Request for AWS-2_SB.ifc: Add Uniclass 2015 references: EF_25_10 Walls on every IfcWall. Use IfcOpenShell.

First a look at what the model holds.

```python
import ifcopenshell

model = ifcopenshell.open("AWS-2_SB.ifc")
print(model.schema)
print("classifications:", [c.Name for c in model.by_type("IfcClassification")])
for ifc_class in ("IfcDoor", "IfcRoof", "IfcStair", "IfcWall", "IfcWindow"):
    print(ifc_class, len(model.by_type(ifc_class)))
```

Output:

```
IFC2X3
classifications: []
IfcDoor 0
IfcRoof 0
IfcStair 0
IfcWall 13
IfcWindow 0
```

```python
import ifcopenshell
import ifcopenshell.api.classification

model = ifcopenshell.open("AWS-2_SB.ifc")

# IFC2X3 requires Source and Edition and has no link from the project to the system.
system = model.create_entity("IfcClassification", Source="NBS", Edition="2015", Name="Uniclass 2015")

codes = {
    "IfcWall": ("EF_25_10", "Walls"),
}
for ifc_class, (code, name) in codes.items():
    products = model.by_type(ifc_class)
    ifcopenshell.api.classification.add_reference(
        model, products=products, classification=system, identification=code, name=name
    )
    print(code, len(products))

model.write("AWS-2_SB_updated.ifc")
```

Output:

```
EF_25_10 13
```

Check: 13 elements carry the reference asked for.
